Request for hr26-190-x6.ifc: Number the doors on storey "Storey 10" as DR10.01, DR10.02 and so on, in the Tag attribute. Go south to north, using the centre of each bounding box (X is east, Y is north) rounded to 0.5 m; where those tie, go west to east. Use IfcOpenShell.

First a look at what the model holds.

```python
import ifcopenshell
import ifcopenshell.util.element
import ifcopenshell.util.placement

model = ifcopenshell.open("hr26-190-x6.ifc")
print(model.schema)
storey = next(s for s in model.by_type("IfcBuildingStorey") if s.Name == "Storey 10")
doors = [e for e in ifcopenshell.util.element.get_decomposition(storey) if e.is_a("IfcDoor")]
for e in sorted(doors, key=lambda e: e.id()):
    origin = ifcopenshell.util.placement.get_local_placement(e.ObjectPlacement)[:3, 3]
    print(e.id(), e.Tag, e.Name, origin.round(2) + 0.0, sep=" | ")
```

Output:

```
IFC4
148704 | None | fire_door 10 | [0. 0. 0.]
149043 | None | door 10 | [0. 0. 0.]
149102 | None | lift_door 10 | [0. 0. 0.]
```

```python
import ifcopenshell
import ifcopenshell.geom
import ifcopenshell.util.element
import ifcopenshell.util.shape

model = ifcopenshell.open("hr26-190-x6.ifc")
settings = ifcopenshell.geom.settings()
settings.set("use-world-coords", True)


def centre(element):
    shape = ifcopenshell.geom.create_shape(settings, element)
    return ifcopenshell.util.shape.get_bbox_centroid(shape.geometry)


storey = next(s for s in model.by_type("IfcBuildingStorey") if s.Name == "Storey 10")
doors = [e for e in ifcopenshell.util.element.get_decomposition(storey) if e.is_a("IfcDoor")]

# Insertion points can sit at a corner or the storey origin, so sort by the geometry (in metres).
centres = {e: centre(e) for e in doors}
doors.sort(key=lambda e: (round(centres[e][1] / 0.5), centres[e][0]))

for i, e in enumerate(doors, start=1):
    number = f"DR10.{i:02d}"
    e.Tag = number
    print(e.id(), number)

model.write("hr26-190-x6_rev.ifc")
```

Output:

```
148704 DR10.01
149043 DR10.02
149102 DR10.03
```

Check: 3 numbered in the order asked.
